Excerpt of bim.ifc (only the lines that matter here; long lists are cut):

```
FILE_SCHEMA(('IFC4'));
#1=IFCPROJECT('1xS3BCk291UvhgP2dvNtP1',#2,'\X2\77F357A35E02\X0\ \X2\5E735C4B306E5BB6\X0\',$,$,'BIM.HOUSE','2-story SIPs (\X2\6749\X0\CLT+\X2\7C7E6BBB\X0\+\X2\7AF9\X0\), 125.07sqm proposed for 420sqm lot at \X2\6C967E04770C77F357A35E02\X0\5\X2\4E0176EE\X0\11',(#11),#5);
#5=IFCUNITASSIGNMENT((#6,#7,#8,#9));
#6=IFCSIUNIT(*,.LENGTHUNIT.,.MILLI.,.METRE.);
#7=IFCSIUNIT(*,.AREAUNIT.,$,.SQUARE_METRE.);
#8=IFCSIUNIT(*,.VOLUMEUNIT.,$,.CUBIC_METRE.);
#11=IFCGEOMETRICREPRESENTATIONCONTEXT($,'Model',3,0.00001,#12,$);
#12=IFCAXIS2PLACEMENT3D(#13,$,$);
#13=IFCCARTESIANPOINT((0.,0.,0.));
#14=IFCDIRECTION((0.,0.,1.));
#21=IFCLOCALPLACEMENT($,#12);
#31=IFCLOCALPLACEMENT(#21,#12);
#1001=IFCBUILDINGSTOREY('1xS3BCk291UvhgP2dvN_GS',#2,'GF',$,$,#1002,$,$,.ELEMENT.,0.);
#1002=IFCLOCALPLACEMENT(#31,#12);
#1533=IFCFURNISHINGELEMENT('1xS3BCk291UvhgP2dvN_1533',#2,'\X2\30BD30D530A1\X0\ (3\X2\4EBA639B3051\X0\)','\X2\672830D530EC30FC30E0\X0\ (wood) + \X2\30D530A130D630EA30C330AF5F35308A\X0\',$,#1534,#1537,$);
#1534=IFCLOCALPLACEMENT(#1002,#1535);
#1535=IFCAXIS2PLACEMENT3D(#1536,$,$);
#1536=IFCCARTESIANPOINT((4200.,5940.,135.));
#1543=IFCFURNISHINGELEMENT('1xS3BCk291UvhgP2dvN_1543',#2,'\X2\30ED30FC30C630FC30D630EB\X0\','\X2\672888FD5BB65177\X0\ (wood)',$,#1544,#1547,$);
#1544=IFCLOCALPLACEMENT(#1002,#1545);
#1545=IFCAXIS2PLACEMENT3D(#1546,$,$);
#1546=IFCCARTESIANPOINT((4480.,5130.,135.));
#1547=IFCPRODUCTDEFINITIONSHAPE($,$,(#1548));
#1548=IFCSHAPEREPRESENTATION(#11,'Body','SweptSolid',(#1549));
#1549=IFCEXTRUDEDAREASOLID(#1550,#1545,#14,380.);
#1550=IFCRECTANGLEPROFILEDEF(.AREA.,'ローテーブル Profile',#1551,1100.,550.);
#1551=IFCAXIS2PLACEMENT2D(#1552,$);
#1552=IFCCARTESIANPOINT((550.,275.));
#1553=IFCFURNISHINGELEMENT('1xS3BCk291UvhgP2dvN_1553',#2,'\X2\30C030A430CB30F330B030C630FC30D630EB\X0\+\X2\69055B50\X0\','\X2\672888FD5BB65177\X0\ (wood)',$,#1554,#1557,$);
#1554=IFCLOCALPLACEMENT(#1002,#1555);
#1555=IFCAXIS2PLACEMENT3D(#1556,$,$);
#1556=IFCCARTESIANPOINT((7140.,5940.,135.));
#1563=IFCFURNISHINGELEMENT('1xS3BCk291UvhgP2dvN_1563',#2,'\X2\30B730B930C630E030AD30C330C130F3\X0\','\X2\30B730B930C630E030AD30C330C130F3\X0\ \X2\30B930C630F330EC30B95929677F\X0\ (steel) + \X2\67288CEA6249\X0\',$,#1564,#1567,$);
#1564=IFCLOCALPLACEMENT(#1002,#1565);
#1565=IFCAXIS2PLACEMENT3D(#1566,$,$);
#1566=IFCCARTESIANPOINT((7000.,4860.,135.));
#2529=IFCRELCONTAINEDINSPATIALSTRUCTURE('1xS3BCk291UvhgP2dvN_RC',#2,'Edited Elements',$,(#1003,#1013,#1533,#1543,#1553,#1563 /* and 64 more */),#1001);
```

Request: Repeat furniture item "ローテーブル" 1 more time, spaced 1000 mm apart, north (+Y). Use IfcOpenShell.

```python
import numpy as np
import ifcopenshell
import ifcopenshell.api.geometry
import ifcopenshell.api.root
import ifcopenshell.util.element
import ifcopenshell.util.placement
import ifcopenshell.util.unit

model = ifcopenshell.open("bim.ifc")
unit_scale = ifcopenshell.util.unit.calculate_unit_scale(model)


def reuse_history(source, copy):
    """copy_class also copies each property set's owner history, people and application; keep the originals."""
    for rel in copy.IsDefinedBy:
        if rel.is_a("IfcRelDefinesByProperties") and (history := rel.RelatingPropertyDefinition.OwnerHistory):
            rel.RelatingPropertyDefinition.OwnerHistory = source.OwnerHistory
            ifcopenshell.util.element.remove_deep2(model, history)


source = model.by_id(1543)
base = ifcopenshell.util.placement.get_local_placement(source.ObjectPlacement)
step = np.array([0.0, 1.0, 0.0]) * 1 / unit_scale

for i in range(1, 2):
    copy = ifcopenshell.api.root.copy_class(model, product=source)
    copy.Representation = ifcopenshell.util.element.copy_deep(
        model, source.Representation, exclude=["IfcGeometricRepresentationContext", "IfcRepresentationMap"]
    )
    reuse_history(source, copy)
    matrix = base.copy()
    matrix[:3, 3] += i * step
    print("added at", matrix[:3, 3].round(3) + 0.0)
    ifcopenshell.api.geometry.edit_object_placement(model, product=copy, matrix=matrix, is_si=False)

model.write("bim_updated.ifc")
```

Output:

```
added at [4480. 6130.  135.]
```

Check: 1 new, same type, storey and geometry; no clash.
